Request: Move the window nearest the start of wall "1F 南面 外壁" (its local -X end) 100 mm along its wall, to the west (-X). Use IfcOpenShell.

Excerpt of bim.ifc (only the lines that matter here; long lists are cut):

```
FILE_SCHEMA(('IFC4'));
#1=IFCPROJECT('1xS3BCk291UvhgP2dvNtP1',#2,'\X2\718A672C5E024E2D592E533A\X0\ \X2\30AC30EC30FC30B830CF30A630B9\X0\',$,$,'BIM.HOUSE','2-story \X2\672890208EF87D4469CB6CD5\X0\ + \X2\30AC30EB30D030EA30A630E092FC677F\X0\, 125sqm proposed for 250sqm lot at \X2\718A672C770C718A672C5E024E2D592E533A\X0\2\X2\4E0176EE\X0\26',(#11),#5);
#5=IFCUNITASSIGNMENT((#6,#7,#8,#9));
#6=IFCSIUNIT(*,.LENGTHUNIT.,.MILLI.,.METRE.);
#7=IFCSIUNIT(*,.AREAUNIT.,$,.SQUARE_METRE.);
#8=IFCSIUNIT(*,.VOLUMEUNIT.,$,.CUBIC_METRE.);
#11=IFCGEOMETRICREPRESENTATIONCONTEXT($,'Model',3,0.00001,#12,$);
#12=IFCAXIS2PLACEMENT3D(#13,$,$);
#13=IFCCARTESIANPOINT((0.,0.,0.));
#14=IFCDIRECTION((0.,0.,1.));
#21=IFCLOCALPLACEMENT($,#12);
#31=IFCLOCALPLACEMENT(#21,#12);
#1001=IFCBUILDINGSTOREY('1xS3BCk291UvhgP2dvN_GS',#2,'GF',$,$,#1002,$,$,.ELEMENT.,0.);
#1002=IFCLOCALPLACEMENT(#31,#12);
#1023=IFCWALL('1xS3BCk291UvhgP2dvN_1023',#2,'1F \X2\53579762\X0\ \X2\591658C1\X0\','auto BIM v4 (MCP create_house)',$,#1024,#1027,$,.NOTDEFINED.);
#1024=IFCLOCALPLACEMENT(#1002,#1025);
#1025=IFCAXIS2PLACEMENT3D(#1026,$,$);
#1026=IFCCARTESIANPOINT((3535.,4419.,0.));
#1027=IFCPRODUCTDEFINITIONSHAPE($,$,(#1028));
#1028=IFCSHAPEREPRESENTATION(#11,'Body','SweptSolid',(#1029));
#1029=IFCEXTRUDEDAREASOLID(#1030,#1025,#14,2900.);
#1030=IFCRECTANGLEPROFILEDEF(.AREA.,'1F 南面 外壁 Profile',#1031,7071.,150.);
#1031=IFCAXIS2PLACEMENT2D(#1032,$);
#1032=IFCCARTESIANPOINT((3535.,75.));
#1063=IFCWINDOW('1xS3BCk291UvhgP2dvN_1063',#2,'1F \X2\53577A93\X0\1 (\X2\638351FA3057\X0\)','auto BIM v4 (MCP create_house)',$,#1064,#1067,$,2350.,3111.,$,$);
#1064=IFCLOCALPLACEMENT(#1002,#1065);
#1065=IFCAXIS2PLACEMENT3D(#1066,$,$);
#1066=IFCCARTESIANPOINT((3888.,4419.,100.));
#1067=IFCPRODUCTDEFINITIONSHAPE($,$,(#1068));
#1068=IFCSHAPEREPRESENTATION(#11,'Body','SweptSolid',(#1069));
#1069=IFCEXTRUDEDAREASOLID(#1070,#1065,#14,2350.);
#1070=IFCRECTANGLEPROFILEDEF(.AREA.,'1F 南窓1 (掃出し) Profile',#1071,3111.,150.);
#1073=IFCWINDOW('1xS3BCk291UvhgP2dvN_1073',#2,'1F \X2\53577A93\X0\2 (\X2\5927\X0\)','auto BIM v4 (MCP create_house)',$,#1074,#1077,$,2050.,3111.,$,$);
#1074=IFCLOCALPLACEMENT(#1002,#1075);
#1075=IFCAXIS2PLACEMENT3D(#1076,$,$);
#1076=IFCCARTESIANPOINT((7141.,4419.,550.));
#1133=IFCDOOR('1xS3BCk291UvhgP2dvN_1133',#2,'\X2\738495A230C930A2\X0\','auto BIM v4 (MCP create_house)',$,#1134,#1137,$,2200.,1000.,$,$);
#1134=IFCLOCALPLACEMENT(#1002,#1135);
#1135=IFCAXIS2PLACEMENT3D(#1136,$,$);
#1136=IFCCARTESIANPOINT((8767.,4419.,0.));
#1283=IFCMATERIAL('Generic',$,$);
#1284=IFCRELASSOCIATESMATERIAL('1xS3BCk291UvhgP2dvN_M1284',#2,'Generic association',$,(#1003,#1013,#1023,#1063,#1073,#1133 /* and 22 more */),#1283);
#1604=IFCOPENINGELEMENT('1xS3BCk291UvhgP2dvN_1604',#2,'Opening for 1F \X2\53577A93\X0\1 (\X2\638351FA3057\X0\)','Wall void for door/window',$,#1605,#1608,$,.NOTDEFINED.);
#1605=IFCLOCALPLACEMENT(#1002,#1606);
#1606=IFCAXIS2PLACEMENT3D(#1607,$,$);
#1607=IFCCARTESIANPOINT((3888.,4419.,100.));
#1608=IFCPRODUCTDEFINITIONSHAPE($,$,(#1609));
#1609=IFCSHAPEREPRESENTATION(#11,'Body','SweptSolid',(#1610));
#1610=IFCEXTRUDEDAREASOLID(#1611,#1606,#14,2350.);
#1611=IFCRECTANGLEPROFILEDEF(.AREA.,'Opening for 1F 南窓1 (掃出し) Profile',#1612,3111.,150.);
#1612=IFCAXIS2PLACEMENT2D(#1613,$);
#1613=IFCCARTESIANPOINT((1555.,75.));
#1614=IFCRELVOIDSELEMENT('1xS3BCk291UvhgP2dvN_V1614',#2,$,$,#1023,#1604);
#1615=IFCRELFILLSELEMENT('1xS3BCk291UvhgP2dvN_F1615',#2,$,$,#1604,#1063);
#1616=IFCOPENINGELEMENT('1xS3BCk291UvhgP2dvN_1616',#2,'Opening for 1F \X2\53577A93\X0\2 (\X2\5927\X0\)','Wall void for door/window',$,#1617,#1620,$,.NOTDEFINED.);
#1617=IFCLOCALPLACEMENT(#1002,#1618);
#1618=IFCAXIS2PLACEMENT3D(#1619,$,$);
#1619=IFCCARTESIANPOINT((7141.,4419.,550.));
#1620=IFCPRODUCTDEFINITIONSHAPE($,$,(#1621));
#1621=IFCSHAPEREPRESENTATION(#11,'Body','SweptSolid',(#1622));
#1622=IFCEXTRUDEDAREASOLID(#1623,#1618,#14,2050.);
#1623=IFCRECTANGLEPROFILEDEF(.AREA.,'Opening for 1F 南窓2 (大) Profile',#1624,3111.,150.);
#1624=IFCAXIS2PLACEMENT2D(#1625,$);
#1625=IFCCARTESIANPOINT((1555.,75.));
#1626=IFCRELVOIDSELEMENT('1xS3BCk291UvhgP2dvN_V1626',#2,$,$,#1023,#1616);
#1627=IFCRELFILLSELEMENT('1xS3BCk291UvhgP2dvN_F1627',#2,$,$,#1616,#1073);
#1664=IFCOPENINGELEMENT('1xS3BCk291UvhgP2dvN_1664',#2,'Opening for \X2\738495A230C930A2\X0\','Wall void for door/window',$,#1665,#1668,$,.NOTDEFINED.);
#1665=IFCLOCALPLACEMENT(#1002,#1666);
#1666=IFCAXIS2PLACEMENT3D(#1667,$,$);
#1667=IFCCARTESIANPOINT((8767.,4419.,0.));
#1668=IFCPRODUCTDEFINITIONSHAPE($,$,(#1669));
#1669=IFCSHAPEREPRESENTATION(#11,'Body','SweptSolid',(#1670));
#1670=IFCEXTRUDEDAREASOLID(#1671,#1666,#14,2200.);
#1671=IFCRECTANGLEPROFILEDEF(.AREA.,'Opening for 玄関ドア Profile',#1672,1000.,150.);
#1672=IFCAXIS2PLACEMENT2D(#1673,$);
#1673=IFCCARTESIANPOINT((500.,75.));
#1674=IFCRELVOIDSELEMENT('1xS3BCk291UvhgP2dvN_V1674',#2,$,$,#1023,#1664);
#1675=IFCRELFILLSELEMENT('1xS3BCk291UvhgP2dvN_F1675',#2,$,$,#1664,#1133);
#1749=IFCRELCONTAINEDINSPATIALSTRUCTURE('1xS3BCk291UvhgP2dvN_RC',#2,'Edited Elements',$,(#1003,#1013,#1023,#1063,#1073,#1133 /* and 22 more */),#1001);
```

```python
import ifcopenshell
import ifcopenshell.api.geometry
import ifcopenshell.util.placement
import ifcopenshell.util.unit

model = ifcopenshell.open("bim.ifc")
unit_scale = ifcopenshell.util.unit.calculate_unit_scale(model)

window = model.by_guid("1xS3BCk291UvhgP2dvN_1063")
opening = window.FillsVoids[0].RelatingOpeningElement
wall = opening.VoidsElements[0].RelatingBuildingElement

wall_matrix = ifcopenshell.util.placement.get_local_placement(wall.ObjectPlacement)
shift = wall_matrix[:3, 0] * -0.1 / unit_scale
before = ifcopenshell.util.placement.get_local_placement(window.ObjectPlacement)[:3, 3].copy()

# The window is not placed relative to its opening, so move both.
for product in (opening, window):
    matrix = ifcopenshell.util.placement.get_local_placement(product.ObjectPlacement)
    matrix[:3, 3] += shift
    ifcopenshell.api.geometry.edit_object_placement(model, product=product, matrix=matrix, is_si=False)

after = ifcopenshell.util.placement.get_local_placement(window.ObjectPlacement)[:3, 3]
print("window moved by", (after - before).round(3) + 0.0)

model.write("bim-out.ifc")
```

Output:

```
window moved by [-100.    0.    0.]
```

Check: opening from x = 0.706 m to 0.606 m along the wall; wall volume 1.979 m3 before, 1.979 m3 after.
